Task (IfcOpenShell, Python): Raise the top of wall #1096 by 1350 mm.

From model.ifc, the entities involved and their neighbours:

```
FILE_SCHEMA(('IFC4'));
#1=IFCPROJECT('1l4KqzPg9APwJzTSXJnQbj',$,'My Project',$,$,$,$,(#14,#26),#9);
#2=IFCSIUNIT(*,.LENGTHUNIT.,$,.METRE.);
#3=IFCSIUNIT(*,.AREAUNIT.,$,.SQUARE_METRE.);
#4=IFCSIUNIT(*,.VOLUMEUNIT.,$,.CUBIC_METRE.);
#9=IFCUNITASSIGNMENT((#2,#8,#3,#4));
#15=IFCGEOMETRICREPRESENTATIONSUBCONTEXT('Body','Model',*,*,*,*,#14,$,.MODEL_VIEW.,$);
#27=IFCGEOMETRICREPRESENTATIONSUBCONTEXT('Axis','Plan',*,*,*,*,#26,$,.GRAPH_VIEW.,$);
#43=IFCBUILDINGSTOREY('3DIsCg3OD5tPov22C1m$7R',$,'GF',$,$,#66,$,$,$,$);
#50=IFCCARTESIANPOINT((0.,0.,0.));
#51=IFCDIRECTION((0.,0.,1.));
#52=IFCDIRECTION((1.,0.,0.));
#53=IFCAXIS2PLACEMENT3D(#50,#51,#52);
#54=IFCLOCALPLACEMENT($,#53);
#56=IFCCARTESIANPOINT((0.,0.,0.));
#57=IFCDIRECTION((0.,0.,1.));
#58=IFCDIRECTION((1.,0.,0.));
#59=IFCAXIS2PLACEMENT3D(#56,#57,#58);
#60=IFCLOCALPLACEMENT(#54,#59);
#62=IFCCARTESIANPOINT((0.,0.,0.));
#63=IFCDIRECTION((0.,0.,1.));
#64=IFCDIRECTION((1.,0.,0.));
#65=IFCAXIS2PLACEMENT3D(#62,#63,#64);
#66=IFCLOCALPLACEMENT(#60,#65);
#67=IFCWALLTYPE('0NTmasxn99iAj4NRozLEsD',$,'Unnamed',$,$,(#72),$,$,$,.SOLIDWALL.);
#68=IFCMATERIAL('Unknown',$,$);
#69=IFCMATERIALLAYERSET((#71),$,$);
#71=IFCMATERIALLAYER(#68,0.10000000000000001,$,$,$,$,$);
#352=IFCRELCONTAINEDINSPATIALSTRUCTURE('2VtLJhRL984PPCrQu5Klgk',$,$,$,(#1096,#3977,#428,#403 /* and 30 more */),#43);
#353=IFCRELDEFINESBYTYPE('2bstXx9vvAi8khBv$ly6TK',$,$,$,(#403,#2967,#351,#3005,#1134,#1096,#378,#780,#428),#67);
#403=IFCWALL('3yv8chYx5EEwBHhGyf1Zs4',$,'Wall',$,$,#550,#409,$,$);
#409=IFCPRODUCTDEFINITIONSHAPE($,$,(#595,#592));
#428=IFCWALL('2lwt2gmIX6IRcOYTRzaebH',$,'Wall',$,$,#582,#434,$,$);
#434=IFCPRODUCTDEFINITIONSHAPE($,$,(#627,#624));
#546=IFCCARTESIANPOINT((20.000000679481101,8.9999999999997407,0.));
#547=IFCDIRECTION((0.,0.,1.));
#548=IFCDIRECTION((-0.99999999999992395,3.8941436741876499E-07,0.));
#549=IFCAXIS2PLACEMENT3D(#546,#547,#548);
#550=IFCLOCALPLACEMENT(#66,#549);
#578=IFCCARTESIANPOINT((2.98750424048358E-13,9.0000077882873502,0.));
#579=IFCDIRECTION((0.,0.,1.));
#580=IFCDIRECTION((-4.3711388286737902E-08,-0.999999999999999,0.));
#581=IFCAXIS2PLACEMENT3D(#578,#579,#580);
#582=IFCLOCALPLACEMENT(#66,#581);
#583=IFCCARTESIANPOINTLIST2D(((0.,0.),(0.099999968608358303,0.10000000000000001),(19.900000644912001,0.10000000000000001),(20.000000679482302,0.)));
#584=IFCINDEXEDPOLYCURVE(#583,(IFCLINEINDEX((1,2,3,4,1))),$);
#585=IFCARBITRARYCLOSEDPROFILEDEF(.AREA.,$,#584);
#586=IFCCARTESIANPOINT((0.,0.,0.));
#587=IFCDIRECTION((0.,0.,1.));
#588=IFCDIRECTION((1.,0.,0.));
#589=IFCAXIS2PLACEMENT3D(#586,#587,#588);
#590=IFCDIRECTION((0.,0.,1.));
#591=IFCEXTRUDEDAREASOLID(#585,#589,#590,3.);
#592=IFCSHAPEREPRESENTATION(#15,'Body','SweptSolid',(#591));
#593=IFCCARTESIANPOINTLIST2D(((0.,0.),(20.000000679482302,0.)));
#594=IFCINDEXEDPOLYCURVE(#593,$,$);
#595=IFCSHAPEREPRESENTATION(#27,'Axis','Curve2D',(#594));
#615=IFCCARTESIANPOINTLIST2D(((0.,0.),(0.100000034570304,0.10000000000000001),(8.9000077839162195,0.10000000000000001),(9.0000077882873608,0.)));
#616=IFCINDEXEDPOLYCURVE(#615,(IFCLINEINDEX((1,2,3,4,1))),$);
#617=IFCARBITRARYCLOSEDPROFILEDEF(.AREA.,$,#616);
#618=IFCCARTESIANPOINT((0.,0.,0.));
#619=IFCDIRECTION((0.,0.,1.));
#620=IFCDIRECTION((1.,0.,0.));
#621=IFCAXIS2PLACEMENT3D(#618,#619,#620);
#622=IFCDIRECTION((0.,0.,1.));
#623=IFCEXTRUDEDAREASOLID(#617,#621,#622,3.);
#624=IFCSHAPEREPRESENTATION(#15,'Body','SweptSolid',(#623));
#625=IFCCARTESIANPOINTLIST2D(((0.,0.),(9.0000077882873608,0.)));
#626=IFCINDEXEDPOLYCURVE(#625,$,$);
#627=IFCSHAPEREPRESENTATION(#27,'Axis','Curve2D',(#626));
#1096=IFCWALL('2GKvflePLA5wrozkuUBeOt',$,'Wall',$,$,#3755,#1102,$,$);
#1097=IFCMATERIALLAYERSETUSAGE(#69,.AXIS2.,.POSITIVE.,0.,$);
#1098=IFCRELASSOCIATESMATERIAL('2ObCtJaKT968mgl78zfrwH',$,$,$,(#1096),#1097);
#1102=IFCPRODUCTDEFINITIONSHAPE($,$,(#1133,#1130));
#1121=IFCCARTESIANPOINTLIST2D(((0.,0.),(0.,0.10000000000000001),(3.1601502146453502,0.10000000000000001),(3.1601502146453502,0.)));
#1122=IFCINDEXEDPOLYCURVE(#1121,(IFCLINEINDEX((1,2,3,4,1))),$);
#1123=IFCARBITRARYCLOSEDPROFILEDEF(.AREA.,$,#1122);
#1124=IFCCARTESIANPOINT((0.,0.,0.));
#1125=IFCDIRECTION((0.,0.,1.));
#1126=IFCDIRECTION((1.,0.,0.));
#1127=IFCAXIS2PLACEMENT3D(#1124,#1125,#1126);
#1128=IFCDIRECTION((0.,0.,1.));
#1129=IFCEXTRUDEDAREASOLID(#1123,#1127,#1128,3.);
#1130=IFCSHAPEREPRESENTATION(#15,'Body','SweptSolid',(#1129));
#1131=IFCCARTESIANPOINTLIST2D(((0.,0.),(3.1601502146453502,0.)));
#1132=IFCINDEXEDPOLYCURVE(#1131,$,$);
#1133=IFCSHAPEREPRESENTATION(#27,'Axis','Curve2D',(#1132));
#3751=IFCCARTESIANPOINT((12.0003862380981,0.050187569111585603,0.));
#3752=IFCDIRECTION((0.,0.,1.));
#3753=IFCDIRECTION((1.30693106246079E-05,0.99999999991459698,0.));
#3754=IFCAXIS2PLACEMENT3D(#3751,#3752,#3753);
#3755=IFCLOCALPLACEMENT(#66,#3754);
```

```python
import ifcopenshell
import ifcopenshell.geom
import ifcopenshell.util.representation
import ifcopenshell.util.shape

model = ifcopenshell.open("model.ifc")
settings = ifcopenshell.geom.settings()


def volume(element):
    """Net volume in cubic metres, openings subtracted."""
    shape = ifcopenshell.geom.create_shape(settings, element)
    return ifcopenshell.util.shape.get_volume(shape.geometry)


wall = model.by_guid("2GKvflePLA5wrozkuUBeOt")
before = volume(wall)

body = ifcopenshell.util.representation.get_representation(wall, "Model", "Body")
solid = body.Items[0]
old_height = solid.Depth
solid.Depth += 1.35
after = volume(wall)

print(f"height {old_height:g} -> {solid.Depth:g}, volume {before:.3f} -> {after:.3f} m3")

model.write("model_updated.ifc")
```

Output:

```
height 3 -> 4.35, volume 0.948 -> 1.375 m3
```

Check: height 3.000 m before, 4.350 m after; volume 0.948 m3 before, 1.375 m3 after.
